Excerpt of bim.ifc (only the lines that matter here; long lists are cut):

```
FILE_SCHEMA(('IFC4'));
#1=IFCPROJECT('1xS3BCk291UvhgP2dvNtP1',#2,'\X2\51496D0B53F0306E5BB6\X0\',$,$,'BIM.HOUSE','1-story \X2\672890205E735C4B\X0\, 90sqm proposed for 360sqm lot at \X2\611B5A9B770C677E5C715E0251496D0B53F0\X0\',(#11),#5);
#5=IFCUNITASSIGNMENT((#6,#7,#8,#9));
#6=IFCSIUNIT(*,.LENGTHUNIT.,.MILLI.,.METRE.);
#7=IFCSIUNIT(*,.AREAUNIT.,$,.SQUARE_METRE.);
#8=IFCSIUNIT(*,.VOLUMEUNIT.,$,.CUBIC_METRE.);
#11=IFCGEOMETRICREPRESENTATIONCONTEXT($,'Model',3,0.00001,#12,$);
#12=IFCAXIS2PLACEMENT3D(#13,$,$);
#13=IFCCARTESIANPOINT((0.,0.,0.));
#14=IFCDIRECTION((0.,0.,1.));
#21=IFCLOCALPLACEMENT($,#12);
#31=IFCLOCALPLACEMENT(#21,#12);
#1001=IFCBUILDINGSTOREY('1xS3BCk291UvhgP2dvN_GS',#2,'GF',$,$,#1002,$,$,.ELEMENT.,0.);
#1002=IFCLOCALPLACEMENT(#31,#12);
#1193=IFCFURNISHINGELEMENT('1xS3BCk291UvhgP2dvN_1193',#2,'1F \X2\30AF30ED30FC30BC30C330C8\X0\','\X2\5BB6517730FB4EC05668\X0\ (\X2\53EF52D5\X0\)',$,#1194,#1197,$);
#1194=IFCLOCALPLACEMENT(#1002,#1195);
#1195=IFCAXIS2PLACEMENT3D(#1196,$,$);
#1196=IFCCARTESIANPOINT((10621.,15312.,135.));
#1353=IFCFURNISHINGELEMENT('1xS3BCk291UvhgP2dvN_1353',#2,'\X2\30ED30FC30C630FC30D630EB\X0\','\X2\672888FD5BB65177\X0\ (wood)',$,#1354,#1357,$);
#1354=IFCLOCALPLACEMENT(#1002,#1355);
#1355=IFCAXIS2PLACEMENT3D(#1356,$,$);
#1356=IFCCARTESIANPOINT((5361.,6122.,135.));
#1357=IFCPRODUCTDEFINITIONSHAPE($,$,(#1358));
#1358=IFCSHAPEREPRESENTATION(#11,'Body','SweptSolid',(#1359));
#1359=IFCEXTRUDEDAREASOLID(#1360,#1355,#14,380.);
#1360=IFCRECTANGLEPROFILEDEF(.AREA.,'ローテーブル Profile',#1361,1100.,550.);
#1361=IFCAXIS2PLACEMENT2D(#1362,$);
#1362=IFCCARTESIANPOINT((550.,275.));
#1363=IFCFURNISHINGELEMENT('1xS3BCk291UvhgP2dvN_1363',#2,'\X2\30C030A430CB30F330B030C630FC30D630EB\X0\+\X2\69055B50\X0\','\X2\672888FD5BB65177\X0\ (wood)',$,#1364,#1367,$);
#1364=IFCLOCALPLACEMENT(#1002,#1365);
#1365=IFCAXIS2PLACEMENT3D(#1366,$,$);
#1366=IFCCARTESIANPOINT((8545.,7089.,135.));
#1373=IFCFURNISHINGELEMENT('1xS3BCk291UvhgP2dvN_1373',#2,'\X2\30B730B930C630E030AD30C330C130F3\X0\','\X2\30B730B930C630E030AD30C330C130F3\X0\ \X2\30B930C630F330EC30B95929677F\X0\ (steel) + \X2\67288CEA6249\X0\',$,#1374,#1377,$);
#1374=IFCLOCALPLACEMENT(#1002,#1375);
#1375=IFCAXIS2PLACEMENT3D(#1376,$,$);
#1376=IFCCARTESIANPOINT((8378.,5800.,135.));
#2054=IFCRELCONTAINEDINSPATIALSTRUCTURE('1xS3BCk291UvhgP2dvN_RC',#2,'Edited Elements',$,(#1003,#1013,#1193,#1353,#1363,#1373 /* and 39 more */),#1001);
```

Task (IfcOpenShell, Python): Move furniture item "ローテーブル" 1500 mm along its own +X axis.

```python
import ifcopenshell
import ifcopenshell.api.geometry
import ifcopenshell.util.placement

model = ifcopenshell.open("bim.ifc")

item = model.by_guid("1xS3BCk291UvhgP2dvN_1353")
matrix = ifcopenshell.util.placement.get_local_placement(item.ObjectPlacement)
matrix[:3, 3] += matrix[:3, 0] * 1500.0
ifcopenshell.api.geometry.edit_object_placement(model, product=item, matrix=matrix, is_si=False)

print(ifcopenshell.util.placement.get_local_placement(item.ObjectPlacement).round(3) + 0.0)

model.write("bim_rev.ifc")
```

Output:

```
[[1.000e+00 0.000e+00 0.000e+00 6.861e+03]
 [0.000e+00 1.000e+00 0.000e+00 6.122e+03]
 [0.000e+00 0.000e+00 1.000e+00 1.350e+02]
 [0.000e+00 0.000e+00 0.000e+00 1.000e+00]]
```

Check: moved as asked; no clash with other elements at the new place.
